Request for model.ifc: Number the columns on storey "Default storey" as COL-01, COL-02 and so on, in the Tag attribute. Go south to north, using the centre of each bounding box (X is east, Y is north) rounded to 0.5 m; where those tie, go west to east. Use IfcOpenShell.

First a look at what the model holds.

```python
import ifcopenshell
import ifcopenshell.util.element
import ifcopenshell.util.placement

model = ifcopenshell.open("model.ifc")
print(model.schema)
storey = next(s for s in model.by_type("IfcBuildingStorey") if s.Name == "Default storey")
columns = [e for e in ifcopenshell.util.element.get_decomposition(storey) if e.is_a("IfcColumn")]
for e in sorted(columns, key=lambda e: e.id()):
    origin = ifcopenshell.util.placement.get_local_placement(e.ObjectPlacement)[:3, 3]
    print(e.id(), e.Tag, e.Name, origin.round(2) + 0.0, sep=" | ")
```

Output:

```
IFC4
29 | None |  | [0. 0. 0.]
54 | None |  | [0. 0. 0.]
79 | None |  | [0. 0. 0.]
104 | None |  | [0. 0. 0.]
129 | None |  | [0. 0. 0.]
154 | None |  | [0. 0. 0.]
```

```python
import ifcopenshell
import ifcopenshell.geom
import ifcopenshell.util.element
import ifcopenshell.util.shape

model = ifcopenshell.open("model.ifc")
settings = ifcopenshell.geom.settings()
settings.set("use-world-coords", True)


def centre(element):
    shape = ifcopenshell.geom.create_shape(settings, element)
    return ifcopenshell.util.shape.get_bbox_centroid(shape.geometry)


storey = next(s for s in model.by_type("IfcBuildingStorey") if s.Name == "Default storey")
columns = [e for e in ifcopenshell.util.element.get_decomposition(storey) if e.is_a("IfcColumn")]

# Insertion points can sit at a corner or the storey origin, so sort by the geometry (in metres).
centres = {e: centre(e) for e in columns}
columns.sort(key=lambda e: (round(centres[e][1] / 0.5), centres[e][0]))

for i, e in enumerate(columns, start=1):
    number = f"COL-{i:02d}"
    e.Tag = number
    print(e.id(), number)

model.write("model_edited.ifc")
```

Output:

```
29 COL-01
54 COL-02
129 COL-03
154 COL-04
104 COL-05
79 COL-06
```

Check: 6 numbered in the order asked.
